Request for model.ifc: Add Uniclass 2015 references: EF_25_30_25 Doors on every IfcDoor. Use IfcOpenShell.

First a look at what the model holds.

```python
import ifcopenshell

model = ifcopenshell.open("model.ifc")
print(model.schema)
print("classifications:", [c.Name for c in model.by_type("IfcClassification")])
for ifc_class in ("IfcDoor", "IfcRoof", "IfcStair", "IfcWall", "IfcWindow"):
    print(ifc_class, len(model.by_type(ifc_class)))
```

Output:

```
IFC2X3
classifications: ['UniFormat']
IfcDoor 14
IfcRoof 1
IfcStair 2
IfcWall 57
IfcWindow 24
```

```python
import ifcopenshell
import ifcopenshell.api.classification

model = ifcopenshell.open("model.ifc")

# IFC2X3 requires Source and Edition and has no link from the project to the system.
system = model.create_entity("IfcClassification", Source="NBS", Edition="2015", Name="Uniclass 2015")

codes = {
    "IfcDoor": ("EF_25_30_25", "Doors"),
}
for ifc_class, (code, name) in codes.items():
    products = model.by_type(ifc_class)
    ifcopenshell.api.classification.add_reference(
        model, products=products, classification=system, identification=code, name=name
    )
    print(code, len(products))

model.write("model_updated.ifc")
```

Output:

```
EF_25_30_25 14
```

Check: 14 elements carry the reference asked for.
